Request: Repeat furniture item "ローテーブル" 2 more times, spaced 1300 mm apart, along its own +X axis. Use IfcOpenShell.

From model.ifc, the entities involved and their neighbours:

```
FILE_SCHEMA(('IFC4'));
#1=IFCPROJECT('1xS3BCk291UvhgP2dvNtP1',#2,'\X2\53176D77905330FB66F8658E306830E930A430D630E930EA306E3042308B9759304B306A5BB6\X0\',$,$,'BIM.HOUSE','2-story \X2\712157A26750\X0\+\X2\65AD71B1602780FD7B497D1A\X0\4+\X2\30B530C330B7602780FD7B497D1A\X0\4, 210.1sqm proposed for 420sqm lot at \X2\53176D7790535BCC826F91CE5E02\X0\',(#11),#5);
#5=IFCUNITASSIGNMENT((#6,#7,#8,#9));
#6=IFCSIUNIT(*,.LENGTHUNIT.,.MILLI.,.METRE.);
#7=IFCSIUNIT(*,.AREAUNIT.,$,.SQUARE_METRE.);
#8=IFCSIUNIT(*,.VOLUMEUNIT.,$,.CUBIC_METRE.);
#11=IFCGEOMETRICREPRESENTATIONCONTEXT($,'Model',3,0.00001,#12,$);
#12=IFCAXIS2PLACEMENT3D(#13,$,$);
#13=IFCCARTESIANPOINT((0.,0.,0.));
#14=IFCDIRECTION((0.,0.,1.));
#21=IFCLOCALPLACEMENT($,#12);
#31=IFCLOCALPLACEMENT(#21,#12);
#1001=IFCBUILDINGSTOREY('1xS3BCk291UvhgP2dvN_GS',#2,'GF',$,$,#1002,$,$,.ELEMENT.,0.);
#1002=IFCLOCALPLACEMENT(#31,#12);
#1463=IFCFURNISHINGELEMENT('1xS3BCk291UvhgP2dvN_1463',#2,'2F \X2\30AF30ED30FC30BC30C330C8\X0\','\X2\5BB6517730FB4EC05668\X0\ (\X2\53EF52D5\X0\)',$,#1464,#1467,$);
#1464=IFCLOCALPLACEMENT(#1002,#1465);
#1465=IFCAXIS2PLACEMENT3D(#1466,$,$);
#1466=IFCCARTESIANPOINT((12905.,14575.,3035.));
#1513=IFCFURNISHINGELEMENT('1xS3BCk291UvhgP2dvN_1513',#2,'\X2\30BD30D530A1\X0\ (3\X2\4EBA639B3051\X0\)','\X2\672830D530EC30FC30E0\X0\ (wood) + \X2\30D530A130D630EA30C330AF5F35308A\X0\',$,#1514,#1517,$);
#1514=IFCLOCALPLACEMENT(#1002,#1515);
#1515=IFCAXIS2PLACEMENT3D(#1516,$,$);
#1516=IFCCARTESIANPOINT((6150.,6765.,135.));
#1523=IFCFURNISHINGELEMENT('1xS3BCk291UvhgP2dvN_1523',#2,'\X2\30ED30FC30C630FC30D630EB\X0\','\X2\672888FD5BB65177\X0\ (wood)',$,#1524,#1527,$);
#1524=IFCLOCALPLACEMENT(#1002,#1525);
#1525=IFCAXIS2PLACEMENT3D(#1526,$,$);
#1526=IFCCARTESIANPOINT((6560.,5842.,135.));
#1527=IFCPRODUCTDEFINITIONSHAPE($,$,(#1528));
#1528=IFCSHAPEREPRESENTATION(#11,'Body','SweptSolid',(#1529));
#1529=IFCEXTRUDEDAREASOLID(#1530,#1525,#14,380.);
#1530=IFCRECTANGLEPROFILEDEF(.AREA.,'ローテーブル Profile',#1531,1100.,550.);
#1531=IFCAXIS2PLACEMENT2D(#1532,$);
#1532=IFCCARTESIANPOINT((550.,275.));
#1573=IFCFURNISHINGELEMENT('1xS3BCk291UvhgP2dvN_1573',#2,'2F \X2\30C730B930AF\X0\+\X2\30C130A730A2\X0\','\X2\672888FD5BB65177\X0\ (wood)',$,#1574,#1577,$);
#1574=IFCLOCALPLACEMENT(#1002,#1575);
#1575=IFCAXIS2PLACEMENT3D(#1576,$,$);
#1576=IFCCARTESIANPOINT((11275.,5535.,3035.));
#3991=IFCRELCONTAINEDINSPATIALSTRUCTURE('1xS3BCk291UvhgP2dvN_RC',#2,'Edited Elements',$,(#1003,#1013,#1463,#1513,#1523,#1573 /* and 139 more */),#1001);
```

```python
import ifcopenshell
import ifcopenshell.api.geometry
import ifcopenshell.api.root
import ifcopenshell.util.element
import ifcopenshell.util.placement

model = ifcopenshell.open("model.ifc")


def reuse_history(source, copy):
    """copy_class also copies each property set's owner history, people and application; keep the originals."""
    for rel in copy.IsDefinedBy:
        if rel.is_a("IfcRelDefinesByProperties") and (history := rel.RelatingPropertyDefinition.OwnerHistory):
            rel.RelatingPropertyDefinition.OwnerHistory = source.OwnerHistory
            ifcopenshell.util.element.remove_deep2(model, history)


source = model.by_id(1523)
base = ifcopenshell.util.placement.get_local_placement(source.ObjectPlacement)
step = base[:3, 0] * 1300.0

for i in range(1, 3):
    copy = ifcopenshell.api.root.copy_class(model, product=source)
    copy.Representation = ifcopenshell.util.element.copy_deep(
        model, source.Representation, exclude=["IfcGeometricRepresentationContext", "IfcRepresentationMap"]
    )
    reuse_history(source, copy)
    matrix = base.copy()
    matrix[:3, 3] += i * step
    print("added at", matrix[:3, 3].round(3) + 0.0)
    ifcopenshell.api.geometry.edit_object_placement(model, product=copy, matrix=matrix, is_si=False)

model.write("model-out.ifc")
```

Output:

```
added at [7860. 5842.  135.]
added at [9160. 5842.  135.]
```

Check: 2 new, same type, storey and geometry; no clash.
